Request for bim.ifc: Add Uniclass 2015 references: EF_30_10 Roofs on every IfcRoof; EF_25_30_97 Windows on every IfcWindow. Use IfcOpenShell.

First a look at what the model holds.

```python
import ifcopenshell

model = ifcopenshell.open("bim.ifc")
print(model.schema)
print("classifications:", [c.Name for c in model.by_type("IfcClassification")])
for ifc_class in ("IfcDoor", "IfcRoof", "IfcStair", "IfcWall", "IfcWindow"):
    print(ifc_class, len(model.by_type(ifc_class)))
```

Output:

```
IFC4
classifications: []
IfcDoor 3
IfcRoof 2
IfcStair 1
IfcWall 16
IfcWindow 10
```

```python
import ifcopenshell
import ifcopenshell.api.classification

model = ifcopenshell.open("bim.ifc")

system = ifcopenshell.api.classification.add_classification(model, classification="Uniclass 2015")

codes = {
    "IfcRoof": ("EF_30_10", "Roofs"),
    "IfcWindow": ("EF_25_30_97", "Windows"),
}
for ifc_class, (code, name) in codes.items():
    products = model.by_type(ifc_class)
    ifcopenshell.api.classification.add_reference(
        model, products=products, classification=system, identification=code, name=name
    )
    print(code, len(products))

model.write("bim_updated.ifc")
```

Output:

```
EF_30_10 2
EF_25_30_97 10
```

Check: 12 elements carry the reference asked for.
